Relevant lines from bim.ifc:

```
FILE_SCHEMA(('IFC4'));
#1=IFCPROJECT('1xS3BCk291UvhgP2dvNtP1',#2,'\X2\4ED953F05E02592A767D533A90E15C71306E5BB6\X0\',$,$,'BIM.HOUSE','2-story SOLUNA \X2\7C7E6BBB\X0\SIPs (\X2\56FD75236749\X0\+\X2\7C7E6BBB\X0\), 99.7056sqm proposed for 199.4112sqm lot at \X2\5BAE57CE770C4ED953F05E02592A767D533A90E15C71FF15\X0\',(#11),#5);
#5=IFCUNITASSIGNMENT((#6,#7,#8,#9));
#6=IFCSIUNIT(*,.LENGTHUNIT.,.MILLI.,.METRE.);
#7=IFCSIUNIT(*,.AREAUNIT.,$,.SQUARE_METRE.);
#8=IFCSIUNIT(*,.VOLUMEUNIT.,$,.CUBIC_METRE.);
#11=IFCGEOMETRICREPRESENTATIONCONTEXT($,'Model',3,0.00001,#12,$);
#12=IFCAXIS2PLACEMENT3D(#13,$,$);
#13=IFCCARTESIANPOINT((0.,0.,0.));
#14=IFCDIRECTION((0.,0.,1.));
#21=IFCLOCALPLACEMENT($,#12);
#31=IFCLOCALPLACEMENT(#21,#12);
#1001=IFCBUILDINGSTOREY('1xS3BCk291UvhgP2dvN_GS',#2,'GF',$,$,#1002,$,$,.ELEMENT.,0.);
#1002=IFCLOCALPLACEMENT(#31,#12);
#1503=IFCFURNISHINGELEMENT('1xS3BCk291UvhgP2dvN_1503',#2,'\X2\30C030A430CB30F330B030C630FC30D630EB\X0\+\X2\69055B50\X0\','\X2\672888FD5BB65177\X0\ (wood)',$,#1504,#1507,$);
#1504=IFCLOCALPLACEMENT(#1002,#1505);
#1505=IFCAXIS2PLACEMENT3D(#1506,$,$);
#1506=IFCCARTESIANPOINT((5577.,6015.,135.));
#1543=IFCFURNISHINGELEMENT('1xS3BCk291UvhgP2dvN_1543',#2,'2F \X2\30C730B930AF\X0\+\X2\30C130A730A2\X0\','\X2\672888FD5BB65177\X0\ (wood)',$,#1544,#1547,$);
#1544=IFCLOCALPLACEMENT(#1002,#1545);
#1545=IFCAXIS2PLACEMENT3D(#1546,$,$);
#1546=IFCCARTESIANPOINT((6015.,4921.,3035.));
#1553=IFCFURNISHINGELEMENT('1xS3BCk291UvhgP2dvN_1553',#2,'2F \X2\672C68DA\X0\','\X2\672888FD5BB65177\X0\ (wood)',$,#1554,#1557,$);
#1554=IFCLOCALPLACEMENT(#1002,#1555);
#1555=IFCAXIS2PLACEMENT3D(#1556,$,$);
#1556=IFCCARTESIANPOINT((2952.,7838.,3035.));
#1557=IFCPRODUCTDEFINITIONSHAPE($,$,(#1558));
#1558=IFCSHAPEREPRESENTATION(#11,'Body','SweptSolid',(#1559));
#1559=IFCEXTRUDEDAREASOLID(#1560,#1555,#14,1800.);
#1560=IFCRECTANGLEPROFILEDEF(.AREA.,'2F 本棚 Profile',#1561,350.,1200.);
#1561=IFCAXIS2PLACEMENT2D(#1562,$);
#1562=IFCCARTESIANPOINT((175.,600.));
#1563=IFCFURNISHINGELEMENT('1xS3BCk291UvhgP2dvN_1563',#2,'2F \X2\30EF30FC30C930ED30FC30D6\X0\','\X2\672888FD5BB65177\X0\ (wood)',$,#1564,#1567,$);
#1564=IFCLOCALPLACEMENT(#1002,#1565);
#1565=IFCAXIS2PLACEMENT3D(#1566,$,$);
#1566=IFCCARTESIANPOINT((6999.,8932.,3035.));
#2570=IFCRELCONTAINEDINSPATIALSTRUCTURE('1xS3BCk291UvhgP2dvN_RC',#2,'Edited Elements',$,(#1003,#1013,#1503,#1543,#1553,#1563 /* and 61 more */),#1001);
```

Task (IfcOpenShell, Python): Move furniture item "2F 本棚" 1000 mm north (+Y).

```python
import ifcopenshell
import ifcopenshell.api.geometry
import ifcopenshell.util.placement
import ifcopenshell.util.unit

model = ifcopenshell.open("bim.ifc")
unit_scale = ifcopenshell.util.unit.calculate_unit_scale(model)

item = model.by_id(1553)
matrix = ifcopenshell.util.placement.get_local_placement(item.ObjectPlacement)
matrix[1, 3] += 1 / unit_scale
ifcopenshell.api.geometry.edit_object_placement(model, product=item, matrix=matrix, is_si=False)

print(ifcopenshell.util.placement.get_local_placement(item.ObjectPlacement).round(3) + 0.0)

model.write("bim-out.ifc")
```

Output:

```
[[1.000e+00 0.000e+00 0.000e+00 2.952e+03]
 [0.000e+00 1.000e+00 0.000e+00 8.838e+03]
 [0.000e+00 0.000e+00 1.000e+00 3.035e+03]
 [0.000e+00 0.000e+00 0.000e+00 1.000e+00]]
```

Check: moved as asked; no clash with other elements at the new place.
